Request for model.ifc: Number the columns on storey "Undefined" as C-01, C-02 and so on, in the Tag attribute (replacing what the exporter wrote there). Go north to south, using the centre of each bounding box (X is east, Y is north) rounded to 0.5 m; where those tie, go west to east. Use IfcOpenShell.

First a look at what the model holds.

```python
import ifcopenshell
import ifcopenshell.util.element
import ifcopenshell.util.placement

model = ifcopenshell.open("model.ifc")
print(model.schema)
storey = next(s for s in model.by_type("IfcBuildingStorey") if s.Name == "Undefined")
columns = [e for e in ifcopenshell.util.element.get_decomposition(storey) if e.is_a("IfcColumn")]
for e in sorted(columns, key=lambda e: e.id()):
    origin = ifcopenshell.util.placement.get_local_placement(e.ObjectPlacement)[:3, 3]
    print(e.id(), e.Tag, e.Name, origin.round(2) + 0.0, sep=" | ")
```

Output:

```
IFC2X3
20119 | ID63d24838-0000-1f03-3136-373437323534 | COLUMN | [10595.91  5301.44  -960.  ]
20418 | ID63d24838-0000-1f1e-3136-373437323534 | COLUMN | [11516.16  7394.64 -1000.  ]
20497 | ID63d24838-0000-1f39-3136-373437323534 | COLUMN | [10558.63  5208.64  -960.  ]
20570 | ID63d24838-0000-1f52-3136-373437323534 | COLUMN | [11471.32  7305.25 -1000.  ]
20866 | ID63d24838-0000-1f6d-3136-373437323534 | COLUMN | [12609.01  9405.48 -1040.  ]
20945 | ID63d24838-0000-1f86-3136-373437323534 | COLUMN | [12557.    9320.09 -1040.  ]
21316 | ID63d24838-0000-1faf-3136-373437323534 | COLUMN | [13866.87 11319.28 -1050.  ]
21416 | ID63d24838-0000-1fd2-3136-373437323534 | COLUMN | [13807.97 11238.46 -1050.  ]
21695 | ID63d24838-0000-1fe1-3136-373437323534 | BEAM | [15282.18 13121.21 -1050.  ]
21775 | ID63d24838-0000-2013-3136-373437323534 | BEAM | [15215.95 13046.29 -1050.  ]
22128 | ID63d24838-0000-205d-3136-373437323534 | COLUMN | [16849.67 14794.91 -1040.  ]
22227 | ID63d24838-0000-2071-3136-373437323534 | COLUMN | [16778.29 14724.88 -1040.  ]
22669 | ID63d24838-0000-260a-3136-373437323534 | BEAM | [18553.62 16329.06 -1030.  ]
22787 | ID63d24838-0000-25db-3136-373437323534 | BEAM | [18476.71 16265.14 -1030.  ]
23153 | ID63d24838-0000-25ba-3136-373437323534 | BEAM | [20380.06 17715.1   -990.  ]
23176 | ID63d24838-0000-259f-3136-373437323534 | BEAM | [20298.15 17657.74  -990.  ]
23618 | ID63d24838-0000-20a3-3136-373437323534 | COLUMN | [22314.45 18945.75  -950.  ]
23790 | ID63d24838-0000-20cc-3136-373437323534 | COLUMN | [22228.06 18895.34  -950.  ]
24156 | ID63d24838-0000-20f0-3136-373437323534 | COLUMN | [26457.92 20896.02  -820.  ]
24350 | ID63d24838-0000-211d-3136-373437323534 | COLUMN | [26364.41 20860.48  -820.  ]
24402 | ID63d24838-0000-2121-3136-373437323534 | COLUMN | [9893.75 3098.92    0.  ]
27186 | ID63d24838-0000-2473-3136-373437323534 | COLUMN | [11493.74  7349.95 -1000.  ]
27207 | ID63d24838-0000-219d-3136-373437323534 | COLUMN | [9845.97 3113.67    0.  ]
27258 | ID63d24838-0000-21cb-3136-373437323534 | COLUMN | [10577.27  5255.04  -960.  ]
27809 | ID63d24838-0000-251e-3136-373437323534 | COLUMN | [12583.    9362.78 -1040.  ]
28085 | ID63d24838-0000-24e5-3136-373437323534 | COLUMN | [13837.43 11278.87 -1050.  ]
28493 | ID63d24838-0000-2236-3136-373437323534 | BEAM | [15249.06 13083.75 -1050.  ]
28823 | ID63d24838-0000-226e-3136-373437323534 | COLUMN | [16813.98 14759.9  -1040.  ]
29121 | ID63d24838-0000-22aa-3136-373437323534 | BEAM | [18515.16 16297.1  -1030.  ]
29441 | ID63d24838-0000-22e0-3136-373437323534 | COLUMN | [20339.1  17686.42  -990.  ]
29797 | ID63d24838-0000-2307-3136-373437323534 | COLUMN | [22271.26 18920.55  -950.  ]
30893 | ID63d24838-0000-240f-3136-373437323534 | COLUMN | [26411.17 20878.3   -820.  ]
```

```python
import ifcopenshell
import ifcopenshell.geom
import ifcopenshell.util.element
import ifcopenshell.util.shape

model = ifcopenshell.open("model.ifc")
settings = ifcopenshell.geom.settings()
settings.set("use-world-coords", True)


def centre(element):
    shape = ifcopenshell.geom.create_shape(settings, element)
    return ifcopenshell.util.shape.get_bbox_centroid(shape.geometry)


storey = next(s for s in model.by_type("IfcBuildingStorey") if s.Name == "Undefined")
columns = [e for e in ifcopenshell.util.element.get_decomposition(storey) if e.is_a("IfcColumn")]

# Insertion points can sit at a corner or the storey origin, so sort by the geometry (in metres).
centres = {e: centre(e) for e in columns}
columns.sort(key=lambda e: (-round(centres[e][1] / 0.5), centres[e][0]))

for i, e in enumerate(columns, start=1):
    number = f"C-{i:02d}"
    e.Tag = number
    print(e.id(), number)

model.write("model_edited.ifc")
```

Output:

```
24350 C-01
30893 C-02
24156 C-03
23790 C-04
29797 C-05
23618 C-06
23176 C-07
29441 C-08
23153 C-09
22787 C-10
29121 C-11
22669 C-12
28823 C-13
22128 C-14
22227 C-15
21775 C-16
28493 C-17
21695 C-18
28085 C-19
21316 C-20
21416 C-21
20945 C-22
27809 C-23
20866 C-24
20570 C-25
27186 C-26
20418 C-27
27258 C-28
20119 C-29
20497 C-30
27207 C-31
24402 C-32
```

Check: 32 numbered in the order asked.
